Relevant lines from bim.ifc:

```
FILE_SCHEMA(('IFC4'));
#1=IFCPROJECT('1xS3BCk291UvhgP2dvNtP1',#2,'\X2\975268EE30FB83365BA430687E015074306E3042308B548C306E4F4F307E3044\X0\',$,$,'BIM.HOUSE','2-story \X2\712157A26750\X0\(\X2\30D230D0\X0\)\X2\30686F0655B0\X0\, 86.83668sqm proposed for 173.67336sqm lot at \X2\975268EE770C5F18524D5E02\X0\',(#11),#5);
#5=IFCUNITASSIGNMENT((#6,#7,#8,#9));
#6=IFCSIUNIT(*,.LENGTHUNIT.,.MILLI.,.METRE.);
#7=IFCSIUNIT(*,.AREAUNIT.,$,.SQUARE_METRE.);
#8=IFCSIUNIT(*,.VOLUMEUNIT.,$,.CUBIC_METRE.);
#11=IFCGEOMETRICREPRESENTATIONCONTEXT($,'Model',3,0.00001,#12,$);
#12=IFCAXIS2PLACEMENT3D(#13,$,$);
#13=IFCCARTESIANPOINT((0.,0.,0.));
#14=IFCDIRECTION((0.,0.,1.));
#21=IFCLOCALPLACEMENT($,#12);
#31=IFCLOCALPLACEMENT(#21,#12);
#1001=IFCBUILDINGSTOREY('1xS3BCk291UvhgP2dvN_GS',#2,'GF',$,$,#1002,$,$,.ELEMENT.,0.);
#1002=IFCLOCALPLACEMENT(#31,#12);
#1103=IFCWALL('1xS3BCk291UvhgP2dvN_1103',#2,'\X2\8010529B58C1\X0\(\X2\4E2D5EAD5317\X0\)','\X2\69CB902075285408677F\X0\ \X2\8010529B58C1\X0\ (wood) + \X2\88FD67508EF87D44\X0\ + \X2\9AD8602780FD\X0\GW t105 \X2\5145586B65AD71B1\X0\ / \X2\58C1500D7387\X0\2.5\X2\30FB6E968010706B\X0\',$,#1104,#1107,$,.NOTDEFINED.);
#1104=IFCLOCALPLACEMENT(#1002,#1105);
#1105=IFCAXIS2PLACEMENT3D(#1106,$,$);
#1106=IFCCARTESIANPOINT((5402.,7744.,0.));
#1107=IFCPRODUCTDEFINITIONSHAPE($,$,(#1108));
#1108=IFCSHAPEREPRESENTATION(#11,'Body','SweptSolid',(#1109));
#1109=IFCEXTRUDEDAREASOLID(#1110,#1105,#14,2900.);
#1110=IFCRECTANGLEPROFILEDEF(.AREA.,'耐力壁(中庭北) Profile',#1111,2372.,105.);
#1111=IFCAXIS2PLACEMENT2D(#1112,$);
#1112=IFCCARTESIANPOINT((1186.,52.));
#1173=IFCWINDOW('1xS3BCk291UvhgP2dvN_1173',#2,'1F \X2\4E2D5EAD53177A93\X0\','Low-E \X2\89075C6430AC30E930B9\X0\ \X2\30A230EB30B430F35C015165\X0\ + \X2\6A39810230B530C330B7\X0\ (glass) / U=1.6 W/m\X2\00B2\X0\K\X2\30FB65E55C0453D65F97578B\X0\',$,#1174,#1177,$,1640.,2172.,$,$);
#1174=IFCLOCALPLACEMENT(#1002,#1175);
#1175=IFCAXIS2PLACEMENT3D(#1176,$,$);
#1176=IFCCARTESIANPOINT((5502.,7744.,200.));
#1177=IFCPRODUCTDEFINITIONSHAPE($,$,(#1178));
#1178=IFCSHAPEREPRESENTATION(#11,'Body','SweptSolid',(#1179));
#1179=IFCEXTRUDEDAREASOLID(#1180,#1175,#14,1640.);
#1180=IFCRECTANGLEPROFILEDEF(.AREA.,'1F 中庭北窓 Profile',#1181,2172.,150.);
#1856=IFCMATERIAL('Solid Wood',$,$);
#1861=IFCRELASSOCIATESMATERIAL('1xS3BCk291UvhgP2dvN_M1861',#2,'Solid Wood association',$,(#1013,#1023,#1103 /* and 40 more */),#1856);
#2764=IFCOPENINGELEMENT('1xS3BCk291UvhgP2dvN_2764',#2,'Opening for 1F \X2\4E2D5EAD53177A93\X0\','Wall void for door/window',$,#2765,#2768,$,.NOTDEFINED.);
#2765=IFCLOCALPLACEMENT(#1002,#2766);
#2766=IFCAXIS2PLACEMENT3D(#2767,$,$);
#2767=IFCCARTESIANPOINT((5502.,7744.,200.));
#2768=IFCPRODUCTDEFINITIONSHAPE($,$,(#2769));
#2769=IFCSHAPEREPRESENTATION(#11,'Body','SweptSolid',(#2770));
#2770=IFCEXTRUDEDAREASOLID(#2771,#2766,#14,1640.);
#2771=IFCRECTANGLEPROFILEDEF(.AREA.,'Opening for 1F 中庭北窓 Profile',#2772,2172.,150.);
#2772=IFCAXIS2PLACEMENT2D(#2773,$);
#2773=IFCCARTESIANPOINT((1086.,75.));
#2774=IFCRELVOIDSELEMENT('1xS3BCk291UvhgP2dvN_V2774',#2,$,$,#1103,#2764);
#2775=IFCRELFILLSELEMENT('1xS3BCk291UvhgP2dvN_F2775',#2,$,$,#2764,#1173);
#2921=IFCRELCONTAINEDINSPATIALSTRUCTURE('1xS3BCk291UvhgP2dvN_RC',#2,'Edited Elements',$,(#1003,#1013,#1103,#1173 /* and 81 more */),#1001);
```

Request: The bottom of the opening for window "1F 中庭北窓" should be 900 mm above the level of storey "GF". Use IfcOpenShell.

```python
import numpy as np
import ifcopenshell
import ifcopenshell.api.geometry
import ifcopenshell.geom
import ifcopenshell.util.element
import ifcopenshell.util.placement
import ifcopenshell.util.shape
import ifcopenshell.util.unit

model = ifcopenshell.open("bim.ifc")
unit_scale = ifcopenshell.util.unit.calculate_unit_scale(model)

window = model.by_id(1173)
opening = window.FillsVoids[0].RelatingOpeningElement
storey = ifcopenshell.util.element.get_container(window, ifc_class="IfcBuildingStorey")
level = ifcopenshell.util.placement.get_local_placement(storey.ObjectPlacement)[2, 3]

# The opening's origin need not be at the sill, so measure its lowest point.
shape = ifcopenshell.geom.create_shape(ifcopenshell.geom.settings(), opening)
bottom = ifcopenshell.util.shape.get_shape_bottom_elevation(shape, shape.geometry) / unit_scale
dz = level + 900.0 - bottom

shift = np.array([0.0, 0.0, dz])
# The window is not placed relative to its opening, so move both.
for product in (opening, window):
    matrix = ifcopenshell.util.placement.get_local_placement(product.ObjectPlacement)
    matrix[:3, 3] += shift
    ifcopenshell.api.geometry.edit_object_placement(model, product=product, matrix=matrix, is_si=False)

print(f"moved by {dz * unit_scale:+.3f} m")

model.write("bim_updated.ifc")
```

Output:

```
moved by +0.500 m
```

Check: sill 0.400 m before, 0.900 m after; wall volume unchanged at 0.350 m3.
